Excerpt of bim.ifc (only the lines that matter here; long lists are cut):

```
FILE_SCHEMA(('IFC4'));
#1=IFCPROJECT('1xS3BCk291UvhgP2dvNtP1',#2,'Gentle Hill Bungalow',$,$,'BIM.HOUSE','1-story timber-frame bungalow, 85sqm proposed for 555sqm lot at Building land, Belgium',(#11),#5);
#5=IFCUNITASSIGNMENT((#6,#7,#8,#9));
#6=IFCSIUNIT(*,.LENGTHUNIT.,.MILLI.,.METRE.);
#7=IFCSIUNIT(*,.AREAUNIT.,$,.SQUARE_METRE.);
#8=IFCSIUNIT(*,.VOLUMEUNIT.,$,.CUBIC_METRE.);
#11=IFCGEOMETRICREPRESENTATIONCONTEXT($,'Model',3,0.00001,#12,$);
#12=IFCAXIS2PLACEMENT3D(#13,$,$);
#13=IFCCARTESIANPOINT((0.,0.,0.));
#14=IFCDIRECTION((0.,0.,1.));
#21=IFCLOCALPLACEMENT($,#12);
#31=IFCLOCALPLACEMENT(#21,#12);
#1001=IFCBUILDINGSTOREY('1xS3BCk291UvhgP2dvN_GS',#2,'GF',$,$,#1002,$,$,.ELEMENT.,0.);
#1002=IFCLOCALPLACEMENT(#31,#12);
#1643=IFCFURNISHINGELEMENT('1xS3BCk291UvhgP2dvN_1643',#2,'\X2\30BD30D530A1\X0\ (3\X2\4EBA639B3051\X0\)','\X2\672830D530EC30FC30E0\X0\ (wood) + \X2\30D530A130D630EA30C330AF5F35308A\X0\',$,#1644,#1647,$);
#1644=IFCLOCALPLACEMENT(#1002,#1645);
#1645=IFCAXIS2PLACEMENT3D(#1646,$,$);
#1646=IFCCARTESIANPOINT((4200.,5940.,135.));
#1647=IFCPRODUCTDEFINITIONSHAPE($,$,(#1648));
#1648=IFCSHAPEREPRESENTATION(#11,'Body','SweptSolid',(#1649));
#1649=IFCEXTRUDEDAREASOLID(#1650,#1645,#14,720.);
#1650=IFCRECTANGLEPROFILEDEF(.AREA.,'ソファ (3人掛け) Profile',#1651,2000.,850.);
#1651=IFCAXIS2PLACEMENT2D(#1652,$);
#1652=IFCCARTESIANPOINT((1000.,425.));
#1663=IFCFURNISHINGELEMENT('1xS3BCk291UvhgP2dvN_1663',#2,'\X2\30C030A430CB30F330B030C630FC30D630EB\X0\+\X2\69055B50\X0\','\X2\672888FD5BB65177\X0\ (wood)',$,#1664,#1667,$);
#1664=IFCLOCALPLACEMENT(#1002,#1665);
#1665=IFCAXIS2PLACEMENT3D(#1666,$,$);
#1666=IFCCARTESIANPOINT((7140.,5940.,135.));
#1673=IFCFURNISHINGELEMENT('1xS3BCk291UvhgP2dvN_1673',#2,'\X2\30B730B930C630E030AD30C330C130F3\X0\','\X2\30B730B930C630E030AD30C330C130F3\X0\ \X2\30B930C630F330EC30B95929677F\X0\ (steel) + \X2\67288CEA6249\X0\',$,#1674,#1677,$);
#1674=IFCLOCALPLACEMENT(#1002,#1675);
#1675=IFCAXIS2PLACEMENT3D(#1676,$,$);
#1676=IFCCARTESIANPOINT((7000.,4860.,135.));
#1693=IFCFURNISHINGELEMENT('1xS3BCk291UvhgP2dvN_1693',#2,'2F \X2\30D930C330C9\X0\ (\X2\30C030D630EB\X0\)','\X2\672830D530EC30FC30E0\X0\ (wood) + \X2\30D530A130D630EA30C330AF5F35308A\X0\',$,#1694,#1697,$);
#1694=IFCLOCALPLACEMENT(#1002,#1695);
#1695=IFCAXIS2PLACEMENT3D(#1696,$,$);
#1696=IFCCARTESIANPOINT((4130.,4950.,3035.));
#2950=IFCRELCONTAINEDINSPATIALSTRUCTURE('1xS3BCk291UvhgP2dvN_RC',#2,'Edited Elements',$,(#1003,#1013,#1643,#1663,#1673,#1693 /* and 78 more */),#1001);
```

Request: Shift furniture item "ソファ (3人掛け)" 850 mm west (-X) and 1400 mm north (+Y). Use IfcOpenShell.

```python
import ifcopenshell
import ifcopenshell.api.geometry
import ifcopenshell.util.placement
import ifcopenshell.util.unit

model = ifcopenshell.open("bim.ifc")
unit_scale = ifcopenshell.util.unit.calculate_unit_scale(model)

item = model.by_guid("1xS3BCk291UvhgP2dvN_1643")
matrix = ifcopenshell.util.placement.get_local_placement(item.ObjectPlacement)
matrix[0, 3] -= 0.85 / unit_scale
matrix[1, 3] += 1.4 / unit_scale
ifcopenshell.api.geometry.edit_object_placement(model, product=item, matrix=matrix, is_si=False)

print(ifcopenshell.util.placement.get_local_placement(item.ObjectPlacement).round(3) + 0.0)

model.write("bim-out.ifc")
```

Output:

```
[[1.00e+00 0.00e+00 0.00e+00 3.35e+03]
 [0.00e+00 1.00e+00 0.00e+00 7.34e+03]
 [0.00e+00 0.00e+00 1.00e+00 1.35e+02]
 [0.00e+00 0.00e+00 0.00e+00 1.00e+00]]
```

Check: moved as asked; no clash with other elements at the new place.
